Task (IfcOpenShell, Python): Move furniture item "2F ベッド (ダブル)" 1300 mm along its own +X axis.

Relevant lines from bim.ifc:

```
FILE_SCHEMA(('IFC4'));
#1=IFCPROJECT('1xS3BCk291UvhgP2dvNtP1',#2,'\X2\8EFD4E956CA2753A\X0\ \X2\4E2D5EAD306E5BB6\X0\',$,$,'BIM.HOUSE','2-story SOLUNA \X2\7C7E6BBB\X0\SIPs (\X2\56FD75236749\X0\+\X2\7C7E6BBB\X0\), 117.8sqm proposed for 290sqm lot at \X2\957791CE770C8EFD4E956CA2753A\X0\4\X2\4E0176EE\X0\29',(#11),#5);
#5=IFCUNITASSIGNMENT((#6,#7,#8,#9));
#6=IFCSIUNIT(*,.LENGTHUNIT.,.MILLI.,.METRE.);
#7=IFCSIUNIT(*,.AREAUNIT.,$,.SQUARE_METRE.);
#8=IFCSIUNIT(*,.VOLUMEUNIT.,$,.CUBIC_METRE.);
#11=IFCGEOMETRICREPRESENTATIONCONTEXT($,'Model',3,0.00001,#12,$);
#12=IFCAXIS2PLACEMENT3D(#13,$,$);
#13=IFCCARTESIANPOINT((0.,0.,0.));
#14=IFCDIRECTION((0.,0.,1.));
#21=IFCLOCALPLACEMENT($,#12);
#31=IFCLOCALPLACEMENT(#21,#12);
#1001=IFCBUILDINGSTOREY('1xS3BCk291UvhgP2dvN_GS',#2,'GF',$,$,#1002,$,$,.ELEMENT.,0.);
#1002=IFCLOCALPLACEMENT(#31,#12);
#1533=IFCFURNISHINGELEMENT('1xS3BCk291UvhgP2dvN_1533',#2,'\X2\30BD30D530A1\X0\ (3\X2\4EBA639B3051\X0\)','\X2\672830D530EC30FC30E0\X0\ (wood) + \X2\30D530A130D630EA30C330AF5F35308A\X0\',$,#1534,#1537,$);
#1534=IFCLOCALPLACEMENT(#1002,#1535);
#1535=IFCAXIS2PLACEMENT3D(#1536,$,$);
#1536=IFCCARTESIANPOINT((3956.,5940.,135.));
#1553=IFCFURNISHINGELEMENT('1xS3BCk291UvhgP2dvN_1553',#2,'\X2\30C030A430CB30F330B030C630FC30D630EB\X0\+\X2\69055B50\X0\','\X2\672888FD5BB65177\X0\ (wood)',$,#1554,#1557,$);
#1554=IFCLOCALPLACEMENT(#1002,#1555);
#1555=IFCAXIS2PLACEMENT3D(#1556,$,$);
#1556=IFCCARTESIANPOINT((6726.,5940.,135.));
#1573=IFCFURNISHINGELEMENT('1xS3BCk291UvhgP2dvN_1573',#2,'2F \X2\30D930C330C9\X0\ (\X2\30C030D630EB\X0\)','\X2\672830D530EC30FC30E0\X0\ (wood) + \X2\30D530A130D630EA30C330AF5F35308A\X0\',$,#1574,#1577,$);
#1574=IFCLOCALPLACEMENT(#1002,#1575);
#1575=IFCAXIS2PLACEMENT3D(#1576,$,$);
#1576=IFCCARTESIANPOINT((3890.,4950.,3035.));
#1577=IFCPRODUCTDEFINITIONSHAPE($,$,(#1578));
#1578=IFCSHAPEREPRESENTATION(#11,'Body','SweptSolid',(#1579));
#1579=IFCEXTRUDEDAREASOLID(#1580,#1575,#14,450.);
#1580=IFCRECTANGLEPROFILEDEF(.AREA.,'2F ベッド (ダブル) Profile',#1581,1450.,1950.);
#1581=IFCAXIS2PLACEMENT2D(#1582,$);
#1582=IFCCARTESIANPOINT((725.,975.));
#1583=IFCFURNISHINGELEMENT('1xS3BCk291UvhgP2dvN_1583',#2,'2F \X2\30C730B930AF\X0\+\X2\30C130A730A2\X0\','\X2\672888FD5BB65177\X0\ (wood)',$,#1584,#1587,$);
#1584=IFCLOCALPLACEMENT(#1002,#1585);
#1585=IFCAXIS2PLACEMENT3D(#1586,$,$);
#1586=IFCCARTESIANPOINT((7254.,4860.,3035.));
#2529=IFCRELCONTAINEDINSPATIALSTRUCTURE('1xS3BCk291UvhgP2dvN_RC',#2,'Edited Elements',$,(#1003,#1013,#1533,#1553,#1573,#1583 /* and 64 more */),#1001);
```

```python
import ifcopenshell
import ifcopenshell.api.geometry
import ifcopenshell.util.placement
import ifcopenshell.util.unit

model = ifcopenshell.open("bim.ifc")
unit_scale = ifcopenshell.util.unit.calculate_unit_scale(model)

item = model.by_guid("1xS3BCk291UvhgP2dvN_1573")
matrix = ifcopenshell.util.placement.get_local_placement(item.ObjectPlacement)
matrix[:3, 3] += matrix[:3, 0] * 1.3 / unit_scale
ifcopenshell.api.geometry.edit_object_placement(model, product=item, matrix=matrix, is_si=False)

print(ifcopenshell.util.placement.get_local_placement(item.ObjectPlacement).round(3) + 0.0)

model.write("bim_updated.ifc")
```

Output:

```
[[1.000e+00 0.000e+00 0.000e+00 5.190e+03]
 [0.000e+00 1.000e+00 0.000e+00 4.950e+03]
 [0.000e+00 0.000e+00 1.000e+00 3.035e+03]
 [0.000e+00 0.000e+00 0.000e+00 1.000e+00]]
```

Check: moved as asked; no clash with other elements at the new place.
